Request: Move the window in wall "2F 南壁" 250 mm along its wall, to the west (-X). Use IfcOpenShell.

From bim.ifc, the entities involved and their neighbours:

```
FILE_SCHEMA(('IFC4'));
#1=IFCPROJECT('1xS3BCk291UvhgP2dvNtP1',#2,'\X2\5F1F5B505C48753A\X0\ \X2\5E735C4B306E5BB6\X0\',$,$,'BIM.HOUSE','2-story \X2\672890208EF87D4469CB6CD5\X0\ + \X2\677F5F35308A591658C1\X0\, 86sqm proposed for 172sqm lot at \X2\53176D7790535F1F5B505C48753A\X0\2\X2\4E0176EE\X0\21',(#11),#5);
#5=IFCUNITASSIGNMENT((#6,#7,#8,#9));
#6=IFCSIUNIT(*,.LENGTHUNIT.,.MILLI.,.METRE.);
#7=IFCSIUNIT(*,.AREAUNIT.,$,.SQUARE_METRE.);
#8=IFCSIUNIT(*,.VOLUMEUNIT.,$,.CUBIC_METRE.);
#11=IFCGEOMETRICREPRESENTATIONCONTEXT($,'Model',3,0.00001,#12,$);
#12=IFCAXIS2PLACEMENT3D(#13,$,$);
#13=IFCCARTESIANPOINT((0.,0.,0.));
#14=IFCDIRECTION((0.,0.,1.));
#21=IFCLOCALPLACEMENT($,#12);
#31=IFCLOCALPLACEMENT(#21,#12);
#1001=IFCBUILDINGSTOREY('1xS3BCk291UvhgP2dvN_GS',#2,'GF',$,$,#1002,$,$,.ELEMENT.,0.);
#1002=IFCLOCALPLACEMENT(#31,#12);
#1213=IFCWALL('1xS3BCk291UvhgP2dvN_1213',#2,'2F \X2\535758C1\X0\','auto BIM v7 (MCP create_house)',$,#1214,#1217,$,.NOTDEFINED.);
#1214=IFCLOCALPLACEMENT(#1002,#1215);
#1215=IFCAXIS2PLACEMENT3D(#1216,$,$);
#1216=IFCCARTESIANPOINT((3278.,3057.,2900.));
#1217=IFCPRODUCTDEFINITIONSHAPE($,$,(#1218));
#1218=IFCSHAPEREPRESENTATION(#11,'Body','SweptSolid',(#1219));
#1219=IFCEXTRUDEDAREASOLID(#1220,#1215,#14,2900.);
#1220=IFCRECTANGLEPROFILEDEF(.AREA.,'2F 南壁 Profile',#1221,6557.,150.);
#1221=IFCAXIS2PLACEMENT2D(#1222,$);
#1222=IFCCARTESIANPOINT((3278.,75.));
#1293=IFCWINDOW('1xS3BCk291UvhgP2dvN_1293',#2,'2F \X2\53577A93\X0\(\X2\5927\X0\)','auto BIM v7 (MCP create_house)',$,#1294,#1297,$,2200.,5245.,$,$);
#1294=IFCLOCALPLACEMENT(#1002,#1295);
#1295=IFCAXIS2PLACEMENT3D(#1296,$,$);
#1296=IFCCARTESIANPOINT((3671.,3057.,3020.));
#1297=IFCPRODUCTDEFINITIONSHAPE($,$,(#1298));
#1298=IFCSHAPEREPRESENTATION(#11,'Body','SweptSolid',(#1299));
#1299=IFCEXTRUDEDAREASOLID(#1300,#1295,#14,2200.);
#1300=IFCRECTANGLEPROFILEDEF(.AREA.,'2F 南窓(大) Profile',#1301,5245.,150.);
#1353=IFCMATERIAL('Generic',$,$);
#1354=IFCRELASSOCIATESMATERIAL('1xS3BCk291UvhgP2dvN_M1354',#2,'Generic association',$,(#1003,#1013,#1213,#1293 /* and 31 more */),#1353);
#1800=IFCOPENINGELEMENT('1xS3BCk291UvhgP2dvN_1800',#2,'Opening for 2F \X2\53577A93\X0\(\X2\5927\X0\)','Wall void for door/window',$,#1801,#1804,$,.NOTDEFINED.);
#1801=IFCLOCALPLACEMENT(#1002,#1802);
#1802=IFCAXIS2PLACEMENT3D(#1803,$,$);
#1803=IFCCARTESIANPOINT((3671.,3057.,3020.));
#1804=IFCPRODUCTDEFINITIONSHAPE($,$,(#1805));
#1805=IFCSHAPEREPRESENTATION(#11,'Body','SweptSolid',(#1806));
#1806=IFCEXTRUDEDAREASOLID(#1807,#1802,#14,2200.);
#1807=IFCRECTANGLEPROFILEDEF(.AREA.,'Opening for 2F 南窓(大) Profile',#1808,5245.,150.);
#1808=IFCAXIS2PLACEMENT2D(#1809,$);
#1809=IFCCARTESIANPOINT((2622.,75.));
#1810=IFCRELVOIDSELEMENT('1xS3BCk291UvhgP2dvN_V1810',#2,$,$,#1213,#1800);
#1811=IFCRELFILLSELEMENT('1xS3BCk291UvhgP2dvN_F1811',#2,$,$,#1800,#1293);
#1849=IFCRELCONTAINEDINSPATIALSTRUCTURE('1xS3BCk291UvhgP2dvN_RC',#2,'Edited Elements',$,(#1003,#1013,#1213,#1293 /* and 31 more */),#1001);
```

```python
import ifcopenshell
import ifcopenshell.api.geometry
import ifcopenshell.util.placement
import ifcopenshell.util.unit

model = ifcopenshell.open("bim.ifc")
unit_scale = ifcopenshell.util.unit.calculate_unit_scale(model)

window = model.by_guid("1xS3BCk291UvhgP2dvN_1293")
opening = window.FillsVoids[0].RelatingOpeningElement
wall = opening.VoidsElements[0].RelatingBuildingElement

wall_matrix = ifcopenshell.util.placement.get_local_placement(wall.ObjectPlacement)
shift = wall_matrix[:3, 0] * -0.25 / unit_scale
before = ifcopenshell.util.placement.get_local_placement(window.ObjectPlacement)[:3, 3].copy()

# The window is not placed relative to its opening, so move both.
for product in (opening, window):
    matrix = ifcopenshell.util.placement.get_local_placement(product.ObjectPlacement)
    matrix[:3, 3] += shift
    ifcopenshell.api.geometry.edit_object_placement(model, product=product, matrix=matrix, is_si=False)

after = ifcopenshell.util.placement.get_local_placement(window.ObjectPlacement)[:3, 3]
print("window moved by", (after - before).round(3) + 0.0)

model.write("bim-out.ifc")
```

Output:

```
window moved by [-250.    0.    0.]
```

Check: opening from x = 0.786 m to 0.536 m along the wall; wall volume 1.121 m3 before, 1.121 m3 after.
